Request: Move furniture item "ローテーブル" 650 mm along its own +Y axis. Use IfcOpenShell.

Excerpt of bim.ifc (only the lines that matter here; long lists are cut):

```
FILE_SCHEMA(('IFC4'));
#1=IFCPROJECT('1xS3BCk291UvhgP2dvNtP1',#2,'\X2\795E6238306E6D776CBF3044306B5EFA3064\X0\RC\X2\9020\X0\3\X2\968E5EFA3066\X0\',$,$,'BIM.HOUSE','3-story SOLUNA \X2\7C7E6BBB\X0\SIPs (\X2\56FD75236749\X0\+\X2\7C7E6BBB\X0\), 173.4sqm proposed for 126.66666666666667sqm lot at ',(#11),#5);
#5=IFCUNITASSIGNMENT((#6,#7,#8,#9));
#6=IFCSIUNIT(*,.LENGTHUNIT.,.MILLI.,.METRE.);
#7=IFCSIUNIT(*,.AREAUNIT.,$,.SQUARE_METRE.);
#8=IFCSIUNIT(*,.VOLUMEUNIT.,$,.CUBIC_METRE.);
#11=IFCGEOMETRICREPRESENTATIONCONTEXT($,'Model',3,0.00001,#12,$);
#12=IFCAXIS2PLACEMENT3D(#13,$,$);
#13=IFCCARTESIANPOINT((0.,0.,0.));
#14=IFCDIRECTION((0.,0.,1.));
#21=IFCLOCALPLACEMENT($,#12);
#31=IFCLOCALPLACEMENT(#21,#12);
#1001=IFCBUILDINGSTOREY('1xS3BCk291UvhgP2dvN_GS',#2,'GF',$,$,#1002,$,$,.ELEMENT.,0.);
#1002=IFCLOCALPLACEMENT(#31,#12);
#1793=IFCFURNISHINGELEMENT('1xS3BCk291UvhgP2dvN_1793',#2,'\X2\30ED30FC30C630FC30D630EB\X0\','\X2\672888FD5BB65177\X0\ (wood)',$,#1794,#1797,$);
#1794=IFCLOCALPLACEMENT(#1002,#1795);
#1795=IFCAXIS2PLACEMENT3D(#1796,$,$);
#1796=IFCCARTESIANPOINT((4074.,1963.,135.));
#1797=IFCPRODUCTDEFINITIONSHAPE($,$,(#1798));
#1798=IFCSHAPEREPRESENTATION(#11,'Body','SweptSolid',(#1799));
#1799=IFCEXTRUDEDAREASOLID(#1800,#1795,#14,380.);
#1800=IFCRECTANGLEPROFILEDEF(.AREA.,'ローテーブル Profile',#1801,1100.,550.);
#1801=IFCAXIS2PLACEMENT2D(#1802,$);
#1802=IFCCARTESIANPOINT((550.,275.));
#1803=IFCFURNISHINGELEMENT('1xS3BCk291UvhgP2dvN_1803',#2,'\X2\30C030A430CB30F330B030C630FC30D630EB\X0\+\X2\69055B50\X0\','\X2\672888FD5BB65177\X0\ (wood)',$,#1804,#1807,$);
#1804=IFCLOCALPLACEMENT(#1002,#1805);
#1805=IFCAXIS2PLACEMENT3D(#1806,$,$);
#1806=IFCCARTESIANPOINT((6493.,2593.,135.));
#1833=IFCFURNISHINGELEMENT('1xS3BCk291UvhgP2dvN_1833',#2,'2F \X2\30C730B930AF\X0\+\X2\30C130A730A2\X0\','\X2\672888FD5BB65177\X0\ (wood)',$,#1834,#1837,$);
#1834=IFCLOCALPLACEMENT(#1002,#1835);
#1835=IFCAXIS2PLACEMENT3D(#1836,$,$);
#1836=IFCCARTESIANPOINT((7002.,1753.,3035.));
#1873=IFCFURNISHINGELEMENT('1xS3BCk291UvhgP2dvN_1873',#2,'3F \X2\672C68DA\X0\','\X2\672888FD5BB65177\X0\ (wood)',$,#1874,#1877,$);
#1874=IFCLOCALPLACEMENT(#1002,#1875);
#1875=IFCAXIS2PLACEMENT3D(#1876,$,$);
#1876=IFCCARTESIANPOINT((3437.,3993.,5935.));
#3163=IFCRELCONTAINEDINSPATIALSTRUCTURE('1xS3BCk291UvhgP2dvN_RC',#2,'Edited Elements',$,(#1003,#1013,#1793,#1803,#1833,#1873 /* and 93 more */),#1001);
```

```python
import ifcopenshell
import ifcopenshell.api.geometry
import ifcopenshell.util.placement
import ifcopenshell.util.unit

model = ifcopenshell.open("bim.ifc")
unit_scale = ifcopenshell.util.unit.calculate_unit_scale(model)

item = model.by_guid("1xS3BCk291UvhgP2dvN_1793")
matrix = ifcopenshell.util.placement.get_local_placement(item.ObjectPlacement)
matrix[:3, 3] += matrix[:3, 1] * 0.65 / unit_scale
ifcopenshell.api.geometry.edit_object_placement(model, product=item, matrix=matrix, is_si=False)

print(ifcopenshell.util.placement.get_local_placement(item.ObjectPlacement).round(3) + 0.0)

model.write("bim_v2.ifc")
```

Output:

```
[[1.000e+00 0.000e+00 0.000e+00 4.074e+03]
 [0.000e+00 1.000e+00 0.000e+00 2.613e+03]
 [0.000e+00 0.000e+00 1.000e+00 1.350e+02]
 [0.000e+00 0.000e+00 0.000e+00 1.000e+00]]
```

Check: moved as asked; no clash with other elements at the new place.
